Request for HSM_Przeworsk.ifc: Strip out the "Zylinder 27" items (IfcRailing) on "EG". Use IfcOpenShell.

First a look at what the model holds.

```python
import ifcopenshell
import ifcopenshell.util.element

model = ifcopenshell.open("HSM_Przeworsk.ifc")
print(model.schema)
storey = next(s for s in model.by_type("IfcBuildingStorey") if s.Name == "EG")
railings = [e for e in ifcopenshell.util.element.get_decomposition(storey) if e.is_a("IfcRailing")]
seen = {}
for e in railings:
    element_type = ifcopenshell.util.element.get_type(e)
    name = element_type.Name if element_type not in (None, e) else None
    seen[name] = seen.get(name, 0) + 1
for name, count in sorted(seen.items(), key=str):
    print(count, "x", name)
```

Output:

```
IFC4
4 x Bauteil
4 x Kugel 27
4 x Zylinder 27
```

```python
import ifcopenshell
import ifcopenshell.api.root
import ifcopenshell.util.element

model = ifcopenshell.open("HSM_Przeworsk.ifc")

storey = next(s for s in model.by_type("IfcBuildingStorey") if s.Name == "EG")
railings = [e for e in ifcopenshell.util.element.get_decomposition(storey) if e.is_a("IfcRailing")]
targets = [e for e in railings if (t := ifcopenshell.util.element.get_type(e)) not in (None, e) and t.Name == "Zylinder 27"]

for e in targets:
    ifcopenshell.api.root.remove_product(model, product=e)
print(len(targets), "removed")

model.write("HSM_Przeworsk_updated.ifc")
```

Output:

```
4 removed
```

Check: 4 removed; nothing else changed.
